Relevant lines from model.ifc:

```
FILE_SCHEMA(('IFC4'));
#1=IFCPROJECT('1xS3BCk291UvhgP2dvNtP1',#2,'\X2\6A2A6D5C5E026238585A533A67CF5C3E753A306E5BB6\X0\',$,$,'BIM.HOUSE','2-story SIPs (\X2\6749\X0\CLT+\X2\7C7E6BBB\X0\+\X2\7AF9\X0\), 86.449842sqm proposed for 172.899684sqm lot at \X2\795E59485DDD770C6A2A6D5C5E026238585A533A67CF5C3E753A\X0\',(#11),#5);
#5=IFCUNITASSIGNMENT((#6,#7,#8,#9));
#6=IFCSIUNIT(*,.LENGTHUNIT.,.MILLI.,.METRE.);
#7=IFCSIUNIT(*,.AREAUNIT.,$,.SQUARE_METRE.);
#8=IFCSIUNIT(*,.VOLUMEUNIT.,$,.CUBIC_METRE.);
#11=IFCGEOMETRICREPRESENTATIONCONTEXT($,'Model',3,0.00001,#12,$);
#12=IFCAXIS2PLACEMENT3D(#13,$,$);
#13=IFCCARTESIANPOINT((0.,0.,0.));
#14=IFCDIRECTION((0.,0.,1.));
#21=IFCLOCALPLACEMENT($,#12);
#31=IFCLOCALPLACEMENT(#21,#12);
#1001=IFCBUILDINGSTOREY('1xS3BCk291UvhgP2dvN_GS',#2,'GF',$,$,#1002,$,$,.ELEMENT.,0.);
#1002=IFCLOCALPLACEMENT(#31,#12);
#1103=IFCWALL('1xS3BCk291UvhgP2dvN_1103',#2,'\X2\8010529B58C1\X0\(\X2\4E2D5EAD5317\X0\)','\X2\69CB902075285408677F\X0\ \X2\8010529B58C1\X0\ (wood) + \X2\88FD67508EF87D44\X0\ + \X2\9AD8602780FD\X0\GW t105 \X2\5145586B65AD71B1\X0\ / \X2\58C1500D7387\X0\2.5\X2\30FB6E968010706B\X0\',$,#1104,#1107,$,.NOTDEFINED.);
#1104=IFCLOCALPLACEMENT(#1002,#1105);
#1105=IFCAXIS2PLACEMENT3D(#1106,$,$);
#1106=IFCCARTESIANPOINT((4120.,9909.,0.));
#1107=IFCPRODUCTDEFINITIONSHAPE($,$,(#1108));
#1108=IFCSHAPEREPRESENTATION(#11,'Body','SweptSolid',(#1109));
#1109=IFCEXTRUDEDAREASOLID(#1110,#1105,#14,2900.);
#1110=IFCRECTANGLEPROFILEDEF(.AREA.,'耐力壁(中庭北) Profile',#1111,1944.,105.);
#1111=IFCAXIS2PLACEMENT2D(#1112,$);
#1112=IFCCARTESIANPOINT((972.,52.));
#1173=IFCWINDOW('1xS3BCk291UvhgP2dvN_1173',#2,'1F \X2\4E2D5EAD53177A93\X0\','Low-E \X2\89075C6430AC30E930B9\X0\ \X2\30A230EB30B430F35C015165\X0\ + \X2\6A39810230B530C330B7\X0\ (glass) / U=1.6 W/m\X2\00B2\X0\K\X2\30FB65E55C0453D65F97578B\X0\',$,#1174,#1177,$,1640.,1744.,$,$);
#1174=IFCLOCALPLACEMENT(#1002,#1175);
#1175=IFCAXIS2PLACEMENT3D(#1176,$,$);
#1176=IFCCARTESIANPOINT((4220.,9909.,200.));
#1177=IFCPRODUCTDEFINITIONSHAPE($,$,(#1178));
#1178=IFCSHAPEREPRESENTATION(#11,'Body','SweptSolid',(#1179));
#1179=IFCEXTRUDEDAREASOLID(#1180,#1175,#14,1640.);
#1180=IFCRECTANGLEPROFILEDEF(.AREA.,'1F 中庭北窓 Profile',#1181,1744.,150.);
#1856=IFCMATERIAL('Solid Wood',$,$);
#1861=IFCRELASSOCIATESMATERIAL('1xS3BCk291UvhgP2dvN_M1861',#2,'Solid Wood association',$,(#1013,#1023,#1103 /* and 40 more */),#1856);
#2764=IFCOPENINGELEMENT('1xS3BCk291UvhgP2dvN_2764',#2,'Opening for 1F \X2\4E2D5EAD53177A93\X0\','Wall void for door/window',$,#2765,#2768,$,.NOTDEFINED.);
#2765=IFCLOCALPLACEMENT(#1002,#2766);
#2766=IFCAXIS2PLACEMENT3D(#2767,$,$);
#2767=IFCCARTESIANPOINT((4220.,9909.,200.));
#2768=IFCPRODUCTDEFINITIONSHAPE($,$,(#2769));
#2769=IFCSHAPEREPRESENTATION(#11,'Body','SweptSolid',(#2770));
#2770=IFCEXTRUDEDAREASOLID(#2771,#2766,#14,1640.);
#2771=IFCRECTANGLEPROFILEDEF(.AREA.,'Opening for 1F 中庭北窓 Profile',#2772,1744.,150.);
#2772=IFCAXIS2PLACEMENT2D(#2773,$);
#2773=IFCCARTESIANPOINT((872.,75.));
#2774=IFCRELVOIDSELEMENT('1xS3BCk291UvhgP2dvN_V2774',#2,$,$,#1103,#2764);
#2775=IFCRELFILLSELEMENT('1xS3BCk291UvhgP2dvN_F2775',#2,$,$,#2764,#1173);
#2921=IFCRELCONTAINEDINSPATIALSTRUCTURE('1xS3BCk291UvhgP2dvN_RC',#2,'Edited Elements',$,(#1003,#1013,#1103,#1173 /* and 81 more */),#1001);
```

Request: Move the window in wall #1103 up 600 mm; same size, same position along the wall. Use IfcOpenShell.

```python
import numpy as np
import ifcopenshell
import ifcopenshell.api.geometry
import ifcopenshell.util.placement
import ifcopenshell.util.unit

model = ifcopenshell.open("model.ifc")
unit_scale = ifcopenshell.util.unit.calculate_unit_scale(model)

window = model.by_id(1173)
opening = window.FillsVoids[0].RelatingOpeningElement
dz = 0.6 / unit_scale

shift = np.array([0.0, 0.0, dz])
# The window is not placed relative to its opening, so move both.
for product in (opening, window):
    matrix = ifcopenshell.util.placement.get_local_placement(product.ObjectPlacement)
    matrix[:3, 3] += shift
    ifcopenshell.api.geometry.edit_object_placement(model, product=product, matrix=matrix, is_si=False)

print(f"moved by {dz * unit_scale:+.3f} m")

model.write("model_edited.ifc")
```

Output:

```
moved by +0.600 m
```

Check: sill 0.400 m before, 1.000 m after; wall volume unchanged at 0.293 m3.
